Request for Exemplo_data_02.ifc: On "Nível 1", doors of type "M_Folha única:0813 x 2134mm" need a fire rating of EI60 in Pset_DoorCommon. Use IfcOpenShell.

First a look at what the model holds.

```python
import ifcopenshell
import ifcopenshell.util.element

model = ifcopenshell.open("Exemplo_data_02.ifc")
print(model.schema)
storey = next(s for s in model.by_type("IfcBuildingStorey") if s.Name == "Nível 1")
doors = [e for e in ifcopenshell.util.element.get_decomposition(storey) if e.is_a("IfcDoor")]
seen = {}
for e in doors:
    element_type = ifcopenshell.util.element.get_type(e)
    key = (element_type.Name if element_type != e and element_type else None, ifcopenshell.util.element.get_pset(e, "Pset_DoorCommon", "FireRating"))
    seen[key] = seen.get(key, 0) + 1
for (name, value), count in sorted(seen.items(), key=str):
    print(count, "x", name, "|", value)
```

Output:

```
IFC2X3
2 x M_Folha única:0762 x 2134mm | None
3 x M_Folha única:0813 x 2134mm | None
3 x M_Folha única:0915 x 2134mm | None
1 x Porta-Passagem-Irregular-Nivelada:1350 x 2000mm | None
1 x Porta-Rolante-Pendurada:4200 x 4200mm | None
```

```python
import ifcopenshell
import ifcopenshell.api.pset
import ifcopenshell.util.element

model = ifcopenshell.open("Exemplo_data_02.ifc")

storey = next(s for s in model.by_type("IfcBuildingStorey") if s.Name == "Nível 1")
doors = [e for e in ifcopenshell.util.element.get_decomposition(storey) if e.is_a("IfcDoor")]

count = 0
for e in doors:
    element_type = ifcopenshell.util.element.get_type(e)
    if element_type in (None, e) or element_type.Name != "M_Folha única:0813 x 2134mm":
        continue
    # add_pset returns the element's existing set when there is one.
    pset = ifcopenshell.api.pset.add_pset(model, product=e, name="Pset_DoorCommon")
    ifcopenshell.api.pset.edit_pset(model, pset=pset, properties={"FireRating": "EI60"})
    count += 1

print(count, "doors updated")

model.write("Exemplo_data_02_v2.ifc")
```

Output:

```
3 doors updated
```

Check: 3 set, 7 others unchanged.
